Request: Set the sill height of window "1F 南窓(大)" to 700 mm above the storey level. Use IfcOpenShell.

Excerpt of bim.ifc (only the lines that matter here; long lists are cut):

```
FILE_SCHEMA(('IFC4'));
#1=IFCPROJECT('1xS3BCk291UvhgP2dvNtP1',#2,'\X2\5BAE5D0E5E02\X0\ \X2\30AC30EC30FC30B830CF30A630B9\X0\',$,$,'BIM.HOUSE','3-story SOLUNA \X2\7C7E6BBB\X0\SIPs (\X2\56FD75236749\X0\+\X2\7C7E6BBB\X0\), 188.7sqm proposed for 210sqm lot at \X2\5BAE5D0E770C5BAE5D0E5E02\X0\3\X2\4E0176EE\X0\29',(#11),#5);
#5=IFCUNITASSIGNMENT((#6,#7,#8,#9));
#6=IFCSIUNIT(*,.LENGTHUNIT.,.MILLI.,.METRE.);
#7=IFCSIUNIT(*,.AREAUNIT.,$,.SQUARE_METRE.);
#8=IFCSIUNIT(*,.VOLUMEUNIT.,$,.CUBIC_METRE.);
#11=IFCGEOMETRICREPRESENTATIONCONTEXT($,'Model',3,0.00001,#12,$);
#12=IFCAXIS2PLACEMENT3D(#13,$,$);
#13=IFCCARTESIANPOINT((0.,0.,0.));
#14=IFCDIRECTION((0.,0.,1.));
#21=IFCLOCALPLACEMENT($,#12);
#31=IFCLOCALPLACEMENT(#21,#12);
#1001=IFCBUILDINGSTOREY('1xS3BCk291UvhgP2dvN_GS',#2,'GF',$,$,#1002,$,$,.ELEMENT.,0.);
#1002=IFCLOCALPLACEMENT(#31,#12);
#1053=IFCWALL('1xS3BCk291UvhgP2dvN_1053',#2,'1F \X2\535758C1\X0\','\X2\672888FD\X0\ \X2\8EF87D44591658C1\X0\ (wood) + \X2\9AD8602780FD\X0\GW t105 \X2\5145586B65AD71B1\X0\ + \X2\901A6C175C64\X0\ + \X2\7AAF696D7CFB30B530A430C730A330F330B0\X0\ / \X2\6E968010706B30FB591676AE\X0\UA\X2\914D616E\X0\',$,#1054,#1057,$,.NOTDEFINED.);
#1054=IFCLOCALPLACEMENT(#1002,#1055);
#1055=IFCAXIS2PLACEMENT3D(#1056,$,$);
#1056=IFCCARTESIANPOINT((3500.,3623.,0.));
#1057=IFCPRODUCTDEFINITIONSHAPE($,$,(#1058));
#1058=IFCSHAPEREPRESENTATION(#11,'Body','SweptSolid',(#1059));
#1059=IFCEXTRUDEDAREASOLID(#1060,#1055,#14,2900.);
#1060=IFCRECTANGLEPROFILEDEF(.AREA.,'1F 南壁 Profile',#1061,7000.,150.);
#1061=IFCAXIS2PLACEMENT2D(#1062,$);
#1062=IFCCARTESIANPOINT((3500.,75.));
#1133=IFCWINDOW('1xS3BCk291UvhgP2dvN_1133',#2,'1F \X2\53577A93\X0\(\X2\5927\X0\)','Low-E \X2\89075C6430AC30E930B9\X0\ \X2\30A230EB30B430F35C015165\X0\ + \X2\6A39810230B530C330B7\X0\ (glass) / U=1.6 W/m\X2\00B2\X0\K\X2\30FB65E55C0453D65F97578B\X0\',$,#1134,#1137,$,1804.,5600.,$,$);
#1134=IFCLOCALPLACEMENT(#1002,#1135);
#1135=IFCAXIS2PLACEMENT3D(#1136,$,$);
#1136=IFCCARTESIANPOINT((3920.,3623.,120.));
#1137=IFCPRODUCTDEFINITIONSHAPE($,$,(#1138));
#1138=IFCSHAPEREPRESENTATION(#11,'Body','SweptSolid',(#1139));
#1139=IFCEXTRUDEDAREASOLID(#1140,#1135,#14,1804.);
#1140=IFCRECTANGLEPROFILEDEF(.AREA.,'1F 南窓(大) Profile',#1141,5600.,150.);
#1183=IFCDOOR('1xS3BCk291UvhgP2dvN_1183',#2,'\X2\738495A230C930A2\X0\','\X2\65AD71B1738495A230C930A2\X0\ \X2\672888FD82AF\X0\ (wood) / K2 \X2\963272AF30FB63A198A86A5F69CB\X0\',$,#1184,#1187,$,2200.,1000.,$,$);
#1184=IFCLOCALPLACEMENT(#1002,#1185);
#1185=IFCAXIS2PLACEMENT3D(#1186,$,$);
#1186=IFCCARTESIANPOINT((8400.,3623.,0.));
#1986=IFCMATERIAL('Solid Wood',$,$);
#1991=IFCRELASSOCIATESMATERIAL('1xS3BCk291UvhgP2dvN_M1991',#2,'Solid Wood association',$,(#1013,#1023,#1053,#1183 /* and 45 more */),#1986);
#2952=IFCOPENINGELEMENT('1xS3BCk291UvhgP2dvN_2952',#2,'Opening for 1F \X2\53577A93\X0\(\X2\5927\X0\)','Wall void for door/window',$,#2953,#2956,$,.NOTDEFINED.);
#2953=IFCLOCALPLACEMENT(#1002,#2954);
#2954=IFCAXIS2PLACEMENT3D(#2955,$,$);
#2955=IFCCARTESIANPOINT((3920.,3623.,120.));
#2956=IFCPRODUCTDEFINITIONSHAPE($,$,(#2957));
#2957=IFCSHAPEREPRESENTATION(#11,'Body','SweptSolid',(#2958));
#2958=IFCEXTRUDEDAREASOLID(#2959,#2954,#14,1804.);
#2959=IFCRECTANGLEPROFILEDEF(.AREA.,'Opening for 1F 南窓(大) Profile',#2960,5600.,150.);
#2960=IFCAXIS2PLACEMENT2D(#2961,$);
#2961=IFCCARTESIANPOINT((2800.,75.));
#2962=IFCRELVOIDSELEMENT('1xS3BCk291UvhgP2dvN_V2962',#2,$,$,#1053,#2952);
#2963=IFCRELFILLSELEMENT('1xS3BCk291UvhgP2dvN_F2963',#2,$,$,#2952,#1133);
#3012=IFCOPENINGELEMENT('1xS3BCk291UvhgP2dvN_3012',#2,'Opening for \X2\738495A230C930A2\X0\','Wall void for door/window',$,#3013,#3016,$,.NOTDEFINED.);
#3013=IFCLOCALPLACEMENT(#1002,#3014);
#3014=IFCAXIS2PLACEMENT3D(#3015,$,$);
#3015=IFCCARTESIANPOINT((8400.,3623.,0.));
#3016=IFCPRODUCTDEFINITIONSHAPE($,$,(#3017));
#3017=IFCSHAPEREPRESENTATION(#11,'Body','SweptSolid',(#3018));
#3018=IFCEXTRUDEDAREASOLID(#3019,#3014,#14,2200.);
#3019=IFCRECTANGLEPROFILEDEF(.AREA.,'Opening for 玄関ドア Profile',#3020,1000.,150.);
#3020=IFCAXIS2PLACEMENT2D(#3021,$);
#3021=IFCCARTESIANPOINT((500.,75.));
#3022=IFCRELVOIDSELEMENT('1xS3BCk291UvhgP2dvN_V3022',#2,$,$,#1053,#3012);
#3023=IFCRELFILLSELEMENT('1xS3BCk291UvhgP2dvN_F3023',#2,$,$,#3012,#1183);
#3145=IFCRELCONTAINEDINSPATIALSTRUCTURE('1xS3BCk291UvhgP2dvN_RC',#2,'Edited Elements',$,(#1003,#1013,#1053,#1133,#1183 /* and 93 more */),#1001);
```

```python
import numpy as np
import ifcopenshell
import ifcopenshell.api.geometry
import ifcopenshell.geom
import ifcopenshell.util.element
import ifcopenshell.util.placement
import ifcopenshell.util.shape
import ifcopenshell.util.unit

model = ifcopenshell.open("bim.ifc")
unit_scale = ifcopenshell.util.unit.calculate_unit_scale(model)

window = model.by_guid("1xS3BCk291UvhgP2dvN_1133")
opening = window.FillsVoids[0].RelatingOpeningElement
storey = ifcopenshell.util.element.get_container(window, ifc_class="IfcBuildingStorey")
level = ifcopenshell.util.placement.get_local_placement(storey.ObjectPlacement)[2, 3]

# The opening's origin need not be at the sill, so measure its lowest point.
shape = ifcopenshell.geom.create_shape(ifcopenshell.geom.settings(), opening)
bottom = ifcopenshell.util.shape.get_shape_bottom_elevation(shape, shape.geometry) / unit_scale
dz = level + 0.7 / unit_scale - bottom

shift = np.array([0.0, 0.0, dz])
# The window is not placed relative to its opening, so move both.
for product in (opening, window):
    matrix = ifcopenshell.util.placement.get_local_placement(product.ObjectPlacement)
    matrix[:3, 3] += shift
    ifcopenshell.api.geometry.edit_object_placement(model, product=product, matrix=matrix, is_si=False)

print(f"moved by {dz * unit_scale:+.3f} m")

model.write("bim_rev.ifc")
```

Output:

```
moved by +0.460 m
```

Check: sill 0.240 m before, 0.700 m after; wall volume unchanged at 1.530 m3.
